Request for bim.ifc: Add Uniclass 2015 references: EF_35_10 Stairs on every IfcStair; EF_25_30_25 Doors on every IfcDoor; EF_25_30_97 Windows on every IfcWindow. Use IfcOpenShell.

First a look at what the model holds.

```python
import ifcopenshell

model = ifcopenshell.open("bim.ifc")
print(model.schema)
print("classifications:", [c.Name for c in model.by_type("IfcClassification")])
for ifc_class in ("IfcDoor", "IfcRoof", "IfcStair", "IfcWall", "IfcWindow"):
    print(ifc_class, len(model.by_type(ifc_class)))
```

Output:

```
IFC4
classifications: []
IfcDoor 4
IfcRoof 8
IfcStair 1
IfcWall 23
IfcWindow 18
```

```python
import ifcopenshell
import ifcopenshell.api.classification

model = ifcopenshell.open("bim.ifc")

system = ifcopenshell.api.classification.add_classification(model, classification="Uniclass 2015")

codes = {
    "IfcStair": ("EF_35_10", "Stairs"),
    "IfcDoor": ("EF_25_30_25", "Doors"),
    "IfcWindow": ("EF_25_30_97", "Windows"),
}
for ifc_class, (code, name) in codes.items():
    products = model.by_type(ifc_class)
    ifcopenshell.api.classification.add_reference(
        model, products=products, classification=system, identification=code, name=name
    )
    print(code, len(products))

model.write("bim_edited.ifc")
```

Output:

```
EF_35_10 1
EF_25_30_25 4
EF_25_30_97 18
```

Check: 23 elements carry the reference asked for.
